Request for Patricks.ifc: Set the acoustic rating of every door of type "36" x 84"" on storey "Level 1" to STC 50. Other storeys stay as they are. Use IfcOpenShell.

First a look at what the model holds.

```python
import ifcopenshell
import ifcopenshell.util.element

model = ifcopenshell.open("Patricks.ifc")
print(model.schema)
storey = next(s for s in model.by_type("IfcBuildingStorey") if s.Name == "Level 1")
doors = [e for e in ifcopenshell.util.element.get_decomposition(storey) if e.is_a("IfcDoor")]
seen = {}
for e in doors:
    element_type = ifcopenshell.util.element.get_type(e)
    key = (element_type.Name if element_type != e and element_type else None, ifcopenshell.util.element.get_pset(e, "Pset_DoorCommon", "AcousticRating"))
    seen[key] = seen.get(key, 0) + 1
for (name, value), count in sorted(seen.items(), key=str):
    print(count, "x", name, "|", value)
```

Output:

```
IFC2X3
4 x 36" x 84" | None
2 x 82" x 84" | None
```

```python
import ifcopenshell
import ifcopenshell.api.pset
import ifcopenshell.util.element

model = ifcopenshell.open("Patricks.ifc")

storey = next(s for s in model.by_type("IfcBuildingStorey") if s.Name == "Level 1")
doors = [e for e in ifcopenshell.util.element.get_decomposition(storey) if e.is_a("IfcDoor")]

count = 0
for e in doors:
    element_type = ifcopenshell.util.element.get_type(e)
    if element_type in (None, e) or element_type.Name != '36" x 84"':
        continue
    # add_pset returns the element's existing set when there is one.
    pset = ifcopenshell.api.pset.add_pset(model, product=e, name="Pset_DoorCommon")
    ifcopenshell.api.pset.edit_pset(model, pset=pset, properties={"AcousticRating": "STC 50"})
    count += 1

print(count, "doors updated")

model.write("Patricks_updated.ifc")
```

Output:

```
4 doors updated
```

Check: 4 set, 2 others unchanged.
